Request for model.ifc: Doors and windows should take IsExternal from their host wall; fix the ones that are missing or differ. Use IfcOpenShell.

First a look at what the model holds.

```python
import ifcopenshell
import ifcopenshell.util.element

model = ifcopenshell.open("model.ifc")
print(model.schema)
seen = {}
for e in model.by_type("IfcDoor") + model.by_type("IfcWindow"):
    if not e.FillsVoids:
        continue
    host = e.FillsVoids[0].RelatingOpeningElement.VoidsElements[0].RelatingBuildingElement
    own = ifcopenshell.util.element.get_pset(e, f"Pset_{e.is_a()[3:].removesuffix('StandardCase')}Common", "IsExternal")
    wall = ifcopenshell.util.element.get_pset(host, "Pset_WallCommon", "IsExternal")
    seen[e.is_a(), own, wall] = seen.get((e.is_a(), own, wall), 0) + 1
for (cls, own, wall), count in sorted(seen.items(), key=str):
    print(count, cls, "IsExternal:", own, "| host wall:", wall)
```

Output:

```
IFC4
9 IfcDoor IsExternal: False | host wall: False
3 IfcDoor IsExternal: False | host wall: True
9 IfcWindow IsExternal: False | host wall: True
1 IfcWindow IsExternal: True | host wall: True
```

```python
import ifcopenshell
import ifcopenshell.api.pset
import ifcopenshell.util.element

model = ifcopenshell.open("model.ifc")

count = 0
for ifc_class, pset_name in (("IfcDoor", "Pset_DoorCommon"), ("IfcWindow", "Pset_WindowCommon")):
    for e in model.by_type(ifc_class):
        if not e.FillsVoids:
            continue
        host = e.FillsVoids[0].RelatingOpeningElement.VoidsElements[0].RelatingBuildingElement
        external = ifcopenshell.util.element.get_pset(host, "Pset_WallCommon", "IsExternal")
        if external is None or ifcopenshell.util.element.get_pset(e, pset_name, "IsExternal") == external:
            continue
        pset = ifcopenshell.api.pset.add_pset(model, product=e, name=pset_name)
        ifcopenshell.api.pset.edit_pset(model, pset=pset, properties={"IsExternal": external})
        count += 1

print(count, "updated")

model.write("model-out.ifc")
```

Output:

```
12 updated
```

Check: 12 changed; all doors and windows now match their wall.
